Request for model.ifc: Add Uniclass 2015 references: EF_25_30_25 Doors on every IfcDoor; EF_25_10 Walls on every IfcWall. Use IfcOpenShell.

First a look at what the model holds.

```python
import ifcopenshell

model = ifcopenshell.open("model.ifc")
print(model.schema)
print("classifications:", [c.Name for c in model.by_type("IfcClassification")])
for ifc_class in ("IfcDoor", "IfcRoof", "IfcStair", "IfcWall", "IfcWindow"):
    print(ifc_class, len(model.by_type(ifc_class)))
```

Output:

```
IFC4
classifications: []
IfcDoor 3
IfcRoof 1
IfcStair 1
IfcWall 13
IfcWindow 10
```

```python
import ifcopenshell
import ifcopenshell.api.classification

model = ifcopenshell.open("model.ifc")

system = ifcopenshell.api.classification.add_classification(model, classification="Uniclass 2015")

codes = {
    "IfcDoor": ("EF_25_30_25", "Doors"),
    "IfcWall": ("EF_25_10", "Walls"),
}
for ifc_class, (code, name) in codes.items():
    products = model.by_type(ifc_class)
    ifcopenshell.api.classification.add_reference(
        model, products=products, classification=system, identification=code, name=name
    )
    print(code, len(products))

model.write("model_updated.ifc")
```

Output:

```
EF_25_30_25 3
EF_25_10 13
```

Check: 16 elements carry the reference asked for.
